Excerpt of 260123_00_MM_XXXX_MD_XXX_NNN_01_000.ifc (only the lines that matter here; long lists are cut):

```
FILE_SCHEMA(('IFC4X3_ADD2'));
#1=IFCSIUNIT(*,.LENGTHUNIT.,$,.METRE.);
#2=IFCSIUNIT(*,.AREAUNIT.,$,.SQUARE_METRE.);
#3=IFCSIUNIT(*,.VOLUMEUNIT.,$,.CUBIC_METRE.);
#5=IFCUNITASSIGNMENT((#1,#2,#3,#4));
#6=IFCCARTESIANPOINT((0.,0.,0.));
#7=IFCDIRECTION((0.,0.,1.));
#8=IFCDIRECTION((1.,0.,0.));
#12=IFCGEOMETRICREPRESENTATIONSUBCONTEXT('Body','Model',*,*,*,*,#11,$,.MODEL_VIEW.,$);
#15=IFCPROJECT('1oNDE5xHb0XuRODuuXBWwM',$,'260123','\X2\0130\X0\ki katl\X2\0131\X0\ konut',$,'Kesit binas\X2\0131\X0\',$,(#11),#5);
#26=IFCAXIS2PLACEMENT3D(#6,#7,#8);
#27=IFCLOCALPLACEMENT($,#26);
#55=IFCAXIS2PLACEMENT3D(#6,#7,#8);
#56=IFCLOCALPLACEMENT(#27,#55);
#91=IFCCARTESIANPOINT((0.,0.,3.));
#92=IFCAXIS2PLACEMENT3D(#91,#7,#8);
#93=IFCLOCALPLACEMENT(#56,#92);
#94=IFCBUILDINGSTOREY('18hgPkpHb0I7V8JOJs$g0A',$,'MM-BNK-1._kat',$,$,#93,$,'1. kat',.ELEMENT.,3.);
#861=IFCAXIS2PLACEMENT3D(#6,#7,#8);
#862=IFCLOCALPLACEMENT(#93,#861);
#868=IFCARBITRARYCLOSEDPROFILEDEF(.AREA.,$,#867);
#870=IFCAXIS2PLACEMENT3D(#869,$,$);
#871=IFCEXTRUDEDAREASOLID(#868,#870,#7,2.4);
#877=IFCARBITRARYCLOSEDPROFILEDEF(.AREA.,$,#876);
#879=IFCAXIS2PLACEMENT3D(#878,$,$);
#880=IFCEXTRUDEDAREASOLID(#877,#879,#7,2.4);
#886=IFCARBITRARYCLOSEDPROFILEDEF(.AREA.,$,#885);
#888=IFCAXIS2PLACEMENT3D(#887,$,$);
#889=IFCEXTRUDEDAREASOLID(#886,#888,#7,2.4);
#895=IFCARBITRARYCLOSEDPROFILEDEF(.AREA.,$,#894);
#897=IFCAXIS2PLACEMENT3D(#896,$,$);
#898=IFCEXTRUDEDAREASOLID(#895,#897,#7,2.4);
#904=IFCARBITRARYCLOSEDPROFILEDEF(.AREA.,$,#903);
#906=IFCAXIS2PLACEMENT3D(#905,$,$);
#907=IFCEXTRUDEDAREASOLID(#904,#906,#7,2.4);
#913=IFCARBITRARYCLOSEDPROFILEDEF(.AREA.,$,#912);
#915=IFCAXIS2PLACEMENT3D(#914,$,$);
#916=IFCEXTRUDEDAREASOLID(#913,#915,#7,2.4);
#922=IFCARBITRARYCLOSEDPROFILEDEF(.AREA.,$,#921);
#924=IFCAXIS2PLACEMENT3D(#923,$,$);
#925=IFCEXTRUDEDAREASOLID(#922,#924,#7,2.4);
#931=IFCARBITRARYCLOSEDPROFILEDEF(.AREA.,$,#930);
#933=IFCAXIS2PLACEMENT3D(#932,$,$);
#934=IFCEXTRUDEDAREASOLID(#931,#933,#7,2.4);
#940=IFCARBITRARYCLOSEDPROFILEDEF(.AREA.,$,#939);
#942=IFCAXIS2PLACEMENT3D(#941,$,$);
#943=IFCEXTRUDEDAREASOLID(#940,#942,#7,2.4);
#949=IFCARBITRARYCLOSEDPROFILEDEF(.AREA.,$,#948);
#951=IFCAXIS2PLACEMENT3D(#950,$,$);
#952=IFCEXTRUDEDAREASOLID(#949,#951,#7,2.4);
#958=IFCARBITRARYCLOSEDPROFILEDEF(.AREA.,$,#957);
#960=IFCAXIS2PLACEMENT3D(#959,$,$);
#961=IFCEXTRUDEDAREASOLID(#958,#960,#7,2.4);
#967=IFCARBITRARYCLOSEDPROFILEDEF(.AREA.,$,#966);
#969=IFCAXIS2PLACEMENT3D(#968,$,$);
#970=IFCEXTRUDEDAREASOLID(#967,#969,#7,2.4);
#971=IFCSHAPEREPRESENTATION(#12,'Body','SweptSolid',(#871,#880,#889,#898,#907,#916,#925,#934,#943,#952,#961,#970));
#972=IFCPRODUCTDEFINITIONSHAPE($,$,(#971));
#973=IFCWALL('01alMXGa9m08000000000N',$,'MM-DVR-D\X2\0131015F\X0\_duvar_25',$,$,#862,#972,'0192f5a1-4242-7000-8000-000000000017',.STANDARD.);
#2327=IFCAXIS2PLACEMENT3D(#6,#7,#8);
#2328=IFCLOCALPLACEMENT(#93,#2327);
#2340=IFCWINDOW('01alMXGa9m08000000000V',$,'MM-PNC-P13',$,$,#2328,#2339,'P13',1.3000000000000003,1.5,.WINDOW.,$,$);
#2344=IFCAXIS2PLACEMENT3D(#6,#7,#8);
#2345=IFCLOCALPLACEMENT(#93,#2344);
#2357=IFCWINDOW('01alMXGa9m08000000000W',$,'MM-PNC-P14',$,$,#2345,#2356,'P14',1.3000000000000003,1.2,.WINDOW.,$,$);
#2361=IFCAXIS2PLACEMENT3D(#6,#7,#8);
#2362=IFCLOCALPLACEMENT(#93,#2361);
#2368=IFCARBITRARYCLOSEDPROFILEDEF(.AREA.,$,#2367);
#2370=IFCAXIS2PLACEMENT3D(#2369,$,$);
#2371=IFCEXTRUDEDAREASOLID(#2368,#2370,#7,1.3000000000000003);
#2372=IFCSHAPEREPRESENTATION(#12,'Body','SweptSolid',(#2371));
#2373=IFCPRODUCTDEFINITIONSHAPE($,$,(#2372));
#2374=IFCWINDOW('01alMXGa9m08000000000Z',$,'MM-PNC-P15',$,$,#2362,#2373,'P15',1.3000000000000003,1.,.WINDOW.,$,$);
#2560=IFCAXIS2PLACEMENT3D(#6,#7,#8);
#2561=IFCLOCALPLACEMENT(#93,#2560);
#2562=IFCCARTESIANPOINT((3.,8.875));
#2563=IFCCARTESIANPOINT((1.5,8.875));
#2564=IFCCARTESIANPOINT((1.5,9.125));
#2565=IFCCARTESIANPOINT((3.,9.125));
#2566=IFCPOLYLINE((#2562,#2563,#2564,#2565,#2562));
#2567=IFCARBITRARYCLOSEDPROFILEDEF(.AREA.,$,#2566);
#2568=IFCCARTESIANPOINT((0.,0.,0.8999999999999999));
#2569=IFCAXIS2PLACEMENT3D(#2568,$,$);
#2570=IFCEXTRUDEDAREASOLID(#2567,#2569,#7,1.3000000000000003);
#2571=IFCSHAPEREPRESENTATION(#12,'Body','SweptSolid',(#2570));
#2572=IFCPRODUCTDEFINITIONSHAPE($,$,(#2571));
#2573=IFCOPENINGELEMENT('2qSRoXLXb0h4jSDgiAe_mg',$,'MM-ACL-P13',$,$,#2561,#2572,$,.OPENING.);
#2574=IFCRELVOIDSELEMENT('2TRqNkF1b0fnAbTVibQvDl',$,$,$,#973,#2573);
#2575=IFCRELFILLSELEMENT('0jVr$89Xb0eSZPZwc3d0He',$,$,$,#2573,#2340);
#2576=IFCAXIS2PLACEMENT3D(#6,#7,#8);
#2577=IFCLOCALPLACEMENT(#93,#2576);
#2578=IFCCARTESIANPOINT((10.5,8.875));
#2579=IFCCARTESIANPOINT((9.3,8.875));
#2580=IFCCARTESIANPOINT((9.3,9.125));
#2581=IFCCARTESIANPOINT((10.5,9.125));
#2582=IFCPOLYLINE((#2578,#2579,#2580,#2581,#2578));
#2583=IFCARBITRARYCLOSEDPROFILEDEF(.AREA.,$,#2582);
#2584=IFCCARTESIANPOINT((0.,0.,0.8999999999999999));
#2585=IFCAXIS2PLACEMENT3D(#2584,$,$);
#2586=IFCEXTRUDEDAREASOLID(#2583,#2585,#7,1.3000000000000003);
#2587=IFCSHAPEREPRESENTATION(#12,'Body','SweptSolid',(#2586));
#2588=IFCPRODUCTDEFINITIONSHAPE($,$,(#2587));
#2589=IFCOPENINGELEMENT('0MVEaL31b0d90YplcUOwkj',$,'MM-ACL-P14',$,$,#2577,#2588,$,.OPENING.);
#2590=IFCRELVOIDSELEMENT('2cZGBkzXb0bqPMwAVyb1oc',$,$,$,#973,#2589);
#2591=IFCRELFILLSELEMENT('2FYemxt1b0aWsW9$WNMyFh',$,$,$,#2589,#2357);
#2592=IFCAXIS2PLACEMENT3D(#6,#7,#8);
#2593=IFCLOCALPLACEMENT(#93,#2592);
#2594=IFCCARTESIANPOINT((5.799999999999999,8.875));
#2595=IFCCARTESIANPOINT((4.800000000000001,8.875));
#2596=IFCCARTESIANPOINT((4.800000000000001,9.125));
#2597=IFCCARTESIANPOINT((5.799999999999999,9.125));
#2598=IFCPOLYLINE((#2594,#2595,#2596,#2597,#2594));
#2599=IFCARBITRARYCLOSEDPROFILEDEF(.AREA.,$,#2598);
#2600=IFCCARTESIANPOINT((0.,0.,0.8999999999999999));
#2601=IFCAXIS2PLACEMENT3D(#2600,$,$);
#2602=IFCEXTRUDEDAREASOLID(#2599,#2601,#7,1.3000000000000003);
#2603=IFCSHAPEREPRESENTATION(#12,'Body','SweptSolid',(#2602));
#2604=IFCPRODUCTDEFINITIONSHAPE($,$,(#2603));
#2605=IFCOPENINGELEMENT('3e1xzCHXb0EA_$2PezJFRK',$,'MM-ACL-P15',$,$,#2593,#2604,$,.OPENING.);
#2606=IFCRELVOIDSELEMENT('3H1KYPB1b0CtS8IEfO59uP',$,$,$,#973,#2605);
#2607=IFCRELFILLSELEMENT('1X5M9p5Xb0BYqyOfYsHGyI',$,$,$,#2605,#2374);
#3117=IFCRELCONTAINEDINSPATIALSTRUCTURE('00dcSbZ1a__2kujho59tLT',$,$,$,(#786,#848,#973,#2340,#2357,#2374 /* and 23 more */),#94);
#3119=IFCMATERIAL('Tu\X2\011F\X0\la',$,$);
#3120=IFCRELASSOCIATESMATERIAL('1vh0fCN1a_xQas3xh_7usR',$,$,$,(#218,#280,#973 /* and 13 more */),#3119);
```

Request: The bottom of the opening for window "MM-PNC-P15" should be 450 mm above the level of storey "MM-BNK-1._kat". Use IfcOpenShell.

```python
import numpy as np
import ifcopenshell
import ifcopenshell.api.geometry
import ifcopenshell.geom
import ifcopenshell.util.element
import ifcopenshell.util.placement
import ifcopenshell.util.shape
import ifcopenshell.util.unit

model = ifcopenshell.open("260123_00_MM_XXXX_MD_XXX_NNN_01_000.ifc")
unit_scale = ifcopenshell.util.unit.calculate_unit_scale(model)

window = model.by_id(2374)
opening = window.FillsVoids[0].RelatingOpeningElement
storey = ifcopenshell.util.element.get_container(window, ifc_class="IfcBuildingStorey")
level = ifcopenshell.util.placement.get_local_placement(storey.ObjectPlacement)[2, 3]

# The opening's origin need not be at the sill, so measure its lowest point.
shape = ifcopenshell.geom.create_shape(ifcopenshell.geom.settings(), opening)
bottom = ifcopenshell.util.shape.get_shape_bottom_elevation(shape, shape.geometry) / unit_scale
dz = level + 0.45 / unit_scale - bottom

shift = np.array([0.0, 0.0, dz])
# The window is not placed relative to its opening, so move both.
for product in (opening, window):
    matrix = ifcopenshell.util.placement.get_local_placement(product.ObjectPlacement)
    matrix[:3, 3] += shift
    ifcopenshell.api.geometry.edit_object_placement(model, product=product, matrix=matrix, is_si=False)

print(f"moved by {dz * unit_scale:+.3f} m")

model.write("260123_00_MM_XXXX_MD_XXX_NNN_01_000_updated.ifc")
```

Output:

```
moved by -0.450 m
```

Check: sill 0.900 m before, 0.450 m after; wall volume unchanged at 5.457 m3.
